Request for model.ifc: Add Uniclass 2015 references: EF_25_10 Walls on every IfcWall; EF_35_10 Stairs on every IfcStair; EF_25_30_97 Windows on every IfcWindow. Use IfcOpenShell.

First a look at what the model holds.

```python
import ifcopenshell

model = ifcopenshell.open("model.ifc")
print(model.schema)
print("classifications:", [c.Name for c in model.by_type("IfcClassification")])
for ifc_class in ("IfcDoor", "IfcRoof", "IfcStair", "IfcWall", "IfcWindow"):
    print(ifc_class, len(model.by_type(ifc_class)))
```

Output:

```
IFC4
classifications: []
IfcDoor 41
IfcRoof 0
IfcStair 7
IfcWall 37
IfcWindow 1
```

```python
import ifcopenshell
import ifcopenshell.api.classification

model = ifcopenshell.open("model.ifc")

system = ifcopenshell.api.classification.add_classification(model, classification="Uniclass 2015")

codes = {
    "IfcWall": ("EF_25_10", "Walls"),
    "IfcStair": ("EF_35_10", "Stairs"),
    "IfcWindow": ("EF_25_30_97", "Windows"),
}
for ifc_class, (code, name) in codes.items():
    products = model.by_type(ifc_class)
    ifcopenshell.api.classification.add_reference(
        model, products=products, classification=system, identification=code, name=name
    )
    print(code, len(products))

model.write("model_edited.ifc")
```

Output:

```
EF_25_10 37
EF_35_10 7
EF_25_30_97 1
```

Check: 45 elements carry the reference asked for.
